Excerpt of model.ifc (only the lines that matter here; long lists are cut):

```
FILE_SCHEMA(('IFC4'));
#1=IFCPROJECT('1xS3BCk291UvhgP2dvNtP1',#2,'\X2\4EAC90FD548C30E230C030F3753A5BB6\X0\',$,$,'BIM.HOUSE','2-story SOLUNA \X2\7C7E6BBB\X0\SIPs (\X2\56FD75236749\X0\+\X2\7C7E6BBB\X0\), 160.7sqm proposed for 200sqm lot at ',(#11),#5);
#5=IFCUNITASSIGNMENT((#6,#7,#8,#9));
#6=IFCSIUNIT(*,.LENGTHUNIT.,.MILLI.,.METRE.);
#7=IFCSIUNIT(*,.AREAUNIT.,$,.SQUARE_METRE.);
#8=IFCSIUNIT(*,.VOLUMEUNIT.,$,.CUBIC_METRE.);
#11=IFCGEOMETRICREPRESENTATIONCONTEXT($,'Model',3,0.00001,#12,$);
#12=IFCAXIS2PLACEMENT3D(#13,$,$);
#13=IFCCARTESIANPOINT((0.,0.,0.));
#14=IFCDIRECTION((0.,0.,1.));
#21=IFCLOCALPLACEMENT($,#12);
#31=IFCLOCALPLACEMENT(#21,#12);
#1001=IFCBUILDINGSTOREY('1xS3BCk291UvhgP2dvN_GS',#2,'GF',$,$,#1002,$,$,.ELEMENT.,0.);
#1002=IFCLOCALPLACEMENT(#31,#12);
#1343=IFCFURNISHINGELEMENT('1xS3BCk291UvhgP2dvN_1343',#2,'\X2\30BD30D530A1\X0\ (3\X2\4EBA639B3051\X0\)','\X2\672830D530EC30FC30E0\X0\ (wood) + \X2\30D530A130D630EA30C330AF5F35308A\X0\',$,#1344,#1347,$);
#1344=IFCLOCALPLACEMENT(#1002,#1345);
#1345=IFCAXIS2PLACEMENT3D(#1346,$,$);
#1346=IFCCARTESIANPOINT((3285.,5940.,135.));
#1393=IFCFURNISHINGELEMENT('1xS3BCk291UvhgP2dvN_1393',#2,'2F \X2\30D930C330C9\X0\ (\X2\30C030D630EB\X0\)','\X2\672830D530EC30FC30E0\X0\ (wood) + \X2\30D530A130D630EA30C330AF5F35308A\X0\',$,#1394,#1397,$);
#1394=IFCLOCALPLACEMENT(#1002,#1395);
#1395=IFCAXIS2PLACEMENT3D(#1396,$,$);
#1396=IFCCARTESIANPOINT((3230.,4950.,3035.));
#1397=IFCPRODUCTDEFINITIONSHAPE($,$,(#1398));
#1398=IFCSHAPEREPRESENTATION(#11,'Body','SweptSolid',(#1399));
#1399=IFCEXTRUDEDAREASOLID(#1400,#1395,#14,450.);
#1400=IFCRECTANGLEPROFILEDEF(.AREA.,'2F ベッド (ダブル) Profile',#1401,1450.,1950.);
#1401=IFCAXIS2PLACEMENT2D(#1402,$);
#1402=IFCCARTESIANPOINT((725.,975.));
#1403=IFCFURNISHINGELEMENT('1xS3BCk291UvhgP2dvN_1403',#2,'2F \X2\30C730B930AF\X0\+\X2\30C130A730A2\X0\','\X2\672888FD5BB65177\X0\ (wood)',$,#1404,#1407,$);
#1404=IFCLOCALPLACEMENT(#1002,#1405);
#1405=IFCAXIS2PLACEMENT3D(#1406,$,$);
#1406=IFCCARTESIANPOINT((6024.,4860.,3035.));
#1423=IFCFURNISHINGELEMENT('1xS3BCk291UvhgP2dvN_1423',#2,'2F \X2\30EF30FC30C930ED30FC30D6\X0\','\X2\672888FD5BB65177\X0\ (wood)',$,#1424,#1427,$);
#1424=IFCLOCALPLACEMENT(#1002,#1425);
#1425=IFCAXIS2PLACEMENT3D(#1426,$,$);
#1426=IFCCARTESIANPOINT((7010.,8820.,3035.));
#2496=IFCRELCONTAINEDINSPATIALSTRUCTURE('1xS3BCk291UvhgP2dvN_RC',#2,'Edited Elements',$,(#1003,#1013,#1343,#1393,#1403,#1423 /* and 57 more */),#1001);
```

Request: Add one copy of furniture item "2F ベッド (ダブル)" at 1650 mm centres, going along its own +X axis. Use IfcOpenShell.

```python
import ifcopenshell
import ifcopenshell.api.geometry
import ifcopenshell.api.root
import ifcopenshell.util.element
import ifcopenshell.util.placement
import ifcopenshell.util.unit

model = ifcopenshell.open("model.ifc")
unit_scale = ifcopenshell.util.unit.calculate_unit_scale(model)


def reuse_history(source, copy):
    """copy_class also copies each property set's owner history, people and application; keep the originals."""
    for rel in copy.IsDefinedBy:
        if rel.is_a("IfcRelDefinesByProperties") and (history := rel.RelatingPropertyDefinition.OwnerHistory):
            rel.RelatingPropertyDefinition.OwnerHistory = source.OwnerHistory
            ifcopenshell.util.element.remove_deep2(model, history)


source = model.by_guid("1xS3BCk291UvhgP2dvN_1393")
base = ifcopenshell.util.placement.get_local_placement(source.ObjectPlacement)
step = base[:3, 0] * 1.65 / unit_scale

for i in range(1, 2):
    copy = ifcopenshell.api.root.copy_class(model, product=source)
    copy.Representation = ifcopenshell.util.element.copy_deep(
        model, source.Representation, exclude=["IfcGeometricRepresentationContext", "IfcRepresentationMap"]
    )
    reuse_history(source, copy)
    matrix = base.copy()
    matrix[:3, 3] += i * step
    print("added at", matrix[:3, 3].round(3) + 0.0)
    ifcopenshell.api.geometry.edit_object_placement(model, product=copy, matrix=matrix, is_si=False)

model.write("model_edited.ifc")
```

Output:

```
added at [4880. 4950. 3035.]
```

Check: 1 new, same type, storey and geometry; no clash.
